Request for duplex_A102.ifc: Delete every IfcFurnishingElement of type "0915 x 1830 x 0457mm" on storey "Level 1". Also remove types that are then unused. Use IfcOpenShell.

First a look at what the model holds.

```python
import ifcopenshell
import ifcopenshell.util.element

model = ifcopenshell.open("duplex_A102.ifc")
print(model.schema)
storey = next(s for s in model.by_type("IfcBuildingStorey") if s.Name == "Level 1")
furniture = [e for e in ifcopenshell.util.element.get_decomposition(storey) if e.is_a("IfcFurnishingElement")]
seen = {}
for e in furniture:
    element_type = ifcopenshell.util.element.get_type(e)
    name = element_type.Name if element_type not in (None, e) else None
    seen[name] = seen.get(name, 0) + 1
for name, count in sorted(seen.items(), key=str):
    print(count, "x", name)
```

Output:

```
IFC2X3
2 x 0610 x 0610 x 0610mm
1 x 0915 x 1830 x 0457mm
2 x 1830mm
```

```python
import ifcopenshell
import ifcopenshell.api.root
import ifcopenshell.util.element

model = ifcopenshell.open("duplex_A102.ifc")

storey = next(s for s in model.by_type("IfcBuildingStorey") if s.Name == "Level 1")
furniture = [e for e in ifcopenshell.util.element.get_decomposition(storey) if e.is_a("IfcFurnishingElement")]
targets = [e for e in furniture if (t := ifcopenshell.util.element.get_type(e)) not in (None, e) and t.Name == "0915 x 1830 x 0457mm"]
types = {ifcopenshell.util.element.get_type(e) for e in targets} - {None, *targets}

for e in targets:
    ifcopenshell.api.root.remove_product(model, product=e)
print(len(targets), "removed")

unused = [t for t in types if not ifcopenshell.util.element.get_types(t)]
for t in unused:
    ifcopenshell.api.root.remove_product(model, product=t)
print(len(unused), "unused types removed")

model.write("duplex_A102_updated.ifc")
```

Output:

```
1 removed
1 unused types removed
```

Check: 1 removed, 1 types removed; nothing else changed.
